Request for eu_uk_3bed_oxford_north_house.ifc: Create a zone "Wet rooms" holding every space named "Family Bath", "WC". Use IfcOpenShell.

First a look at what the model holds.

```python
import ifcopenshell

model = ifcopenshell.open("eu_uk_3bed_oxford_north_house.ifc")
print(model.schema)
seen = {}
for space in model.by_type("IfcSpace"):
    seen[space.LongName] = seen.get(space.LongName, 0) + 1
for name, count in sorted(seen.items(), key=str):
    print(count, "x", name)
print("zones:", [z.Name for z in model.by_type("IfcZone")][:20])
```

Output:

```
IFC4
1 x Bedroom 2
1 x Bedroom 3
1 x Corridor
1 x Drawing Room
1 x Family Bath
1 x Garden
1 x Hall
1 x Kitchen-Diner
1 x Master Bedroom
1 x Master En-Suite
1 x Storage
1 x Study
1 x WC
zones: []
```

```python
import ifcopenshell
import ifcopenshell.api.group
import ifcopenshell.api.root

model = ifcopenshell.open("eu_uk_3bed_oxford_north_house.ifc")

names = {"Family Bath", "WC"}
spaces = [s for s in model.by_type("IfcSpace") if s.LongName in names]

zone = ifcopenshell.api.root.create_entity(model, ifc_class="IfcZone", name="Wet rooms")
ifcopenshell.api.group.assign_group(model, products=spaces, group=zone)
print(len(spaces), "spaces in", zone.Name)

model.write("eu_uk_3bed_oxford_north_house_rev.ifc")
```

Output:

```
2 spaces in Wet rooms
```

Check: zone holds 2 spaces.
